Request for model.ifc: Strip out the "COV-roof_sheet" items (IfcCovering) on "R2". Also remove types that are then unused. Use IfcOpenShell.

First a look at what the model holds.

```python
import ifcopenshell
import ifcopenshell.util.element

model = ifcopenshell.open("model.ifc")
print(model.schema)
storey = next(s for s in model.by_type("IfcBuildingStorey") if s.Name == "R2")
coverings = [e for e in ifcopenshell.util.element.get_decomposition(storey) if e.is_a("IfcCovering")]
seen = {}
for e in coverings:
    element_type = ifcopenshell.util.element.get_type(e)
    name = element_type.Name if element_type not in (None, e) else None
    seen[name] = seen.get(name, 0) + 1
for name, count in sorted(seen.items(), key=str):
    print(count, "x", name)
```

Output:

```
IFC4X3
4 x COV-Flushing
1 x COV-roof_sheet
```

```python
import ifcopenshell
import ifcopenshell.api.root
import ifcopenshell.util.element

model = ifcopenshell.open("model.ifc")

storey = next(s for s in model.by_type("IfcBuildingStorey") if s.Name == "R2")
coverings = [e for e in ifcopenshell.util.element.get_decomposition(storey) if e.is_a("IfcCovering")]
targets = [e for e in coverings if (t := ifcopenshell.util.element.get_type(e)) not in (None, e) and t.Name == "COV-roof_sheet"]
types = {ifcopenshell.util.element.get_type(e) for e in targets} - {None, *targets}

for e in targets:
    ifcopenshell.api.root.remove_product(model, product=e)
print(len(targets), "removed")

unused = [t for t in types if not ifcopenshell.util.element.get_types(t)]
for t in unused:
    ifcopenshell.api.root.remove_product(model, product=t)
print(len(unused), "unused types removed")

model.write("model_edited.ifc")
```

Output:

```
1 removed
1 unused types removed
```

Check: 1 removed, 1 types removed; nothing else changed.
